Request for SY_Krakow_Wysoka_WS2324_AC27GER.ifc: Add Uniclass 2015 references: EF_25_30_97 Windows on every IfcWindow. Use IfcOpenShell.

First a look at what the model holds.

```python
import ifcopenshell

model = ifcopenshell.open("SY_Krakow_Wysoka_WS2324_AC27GER.ifc")
print(model.schema)
print("classifications:", [c.Name for c in model.by_type("IfcClassification")])
for ifc_class in ("IfcDoor", "IfcRoof", "IfcStair", "IfcWall", "IfcWindow"):
    print(ifc_class, len(model.by_type(ifc_class)))
```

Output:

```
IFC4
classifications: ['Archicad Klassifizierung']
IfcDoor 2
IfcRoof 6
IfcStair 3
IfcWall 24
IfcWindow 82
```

```python
import ifcopenshell
import ifcopenshell.api.classification

model = ifcopenshell.open("SY_Krakow_Wysoka_WS2324_AC27GER.ifc")

system = ifcopenshell.api.classification.add_classification(model, classification="Uniclass 2015")

codes = {
    "IfcWindow": ("EF_25_30_97", "Windows"),
}
for ifc_class, (code, name) in codes.items():
    products = model.by_type(ifc_class)
    ifcopenshell.api.classification.add_reference(
        model, products=products, classification=system, identification=code, name=name
    )
    print(code, len(products))

model.write("SY_Krakow_Wysoka_WS2324_AC27GER-out.ifc")
```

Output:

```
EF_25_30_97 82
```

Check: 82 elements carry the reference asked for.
